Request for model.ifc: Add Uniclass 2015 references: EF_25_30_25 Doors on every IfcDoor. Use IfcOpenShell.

First a look at what the model holds.

```python
import ifcopenshell

model = ifcopenshell.open("model.ifc")
print(model.schema)
print("classifications:", [c.Name for c in model.by_type("IfcClassification")])
for ifc_class in ("IfcDoor", "IfcRoof", "IfcStair", "IfcWall", "IfcWindow"):
    print(ifc_class, len(model.by_type(ifc_class)))
```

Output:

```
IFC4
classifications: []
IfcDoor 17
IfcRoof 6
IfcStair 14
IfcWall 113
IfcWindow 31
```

```python
import ifcopenshell
import ifcopenshell.api.classification

model = ifcopenshell.open("model.ifc")

system = ifcopenshell.api.classification.add_classification(model, classification="Uniclass 2015")

codes = {
    "IfcDoor": ("EF_25_30_25", "Doors"),
}
for ifc_class, (code, name) in codes.items():
    products = model.by_type(ifc_class)
    ifcopenshell.api.classification.add_reference(
        model, products=products, classification=system, identification=code, name=name
    )
    print(code, len(products))

model.write("model-out.ifc")
```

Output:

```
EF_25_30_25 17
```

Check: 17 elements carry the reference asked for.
